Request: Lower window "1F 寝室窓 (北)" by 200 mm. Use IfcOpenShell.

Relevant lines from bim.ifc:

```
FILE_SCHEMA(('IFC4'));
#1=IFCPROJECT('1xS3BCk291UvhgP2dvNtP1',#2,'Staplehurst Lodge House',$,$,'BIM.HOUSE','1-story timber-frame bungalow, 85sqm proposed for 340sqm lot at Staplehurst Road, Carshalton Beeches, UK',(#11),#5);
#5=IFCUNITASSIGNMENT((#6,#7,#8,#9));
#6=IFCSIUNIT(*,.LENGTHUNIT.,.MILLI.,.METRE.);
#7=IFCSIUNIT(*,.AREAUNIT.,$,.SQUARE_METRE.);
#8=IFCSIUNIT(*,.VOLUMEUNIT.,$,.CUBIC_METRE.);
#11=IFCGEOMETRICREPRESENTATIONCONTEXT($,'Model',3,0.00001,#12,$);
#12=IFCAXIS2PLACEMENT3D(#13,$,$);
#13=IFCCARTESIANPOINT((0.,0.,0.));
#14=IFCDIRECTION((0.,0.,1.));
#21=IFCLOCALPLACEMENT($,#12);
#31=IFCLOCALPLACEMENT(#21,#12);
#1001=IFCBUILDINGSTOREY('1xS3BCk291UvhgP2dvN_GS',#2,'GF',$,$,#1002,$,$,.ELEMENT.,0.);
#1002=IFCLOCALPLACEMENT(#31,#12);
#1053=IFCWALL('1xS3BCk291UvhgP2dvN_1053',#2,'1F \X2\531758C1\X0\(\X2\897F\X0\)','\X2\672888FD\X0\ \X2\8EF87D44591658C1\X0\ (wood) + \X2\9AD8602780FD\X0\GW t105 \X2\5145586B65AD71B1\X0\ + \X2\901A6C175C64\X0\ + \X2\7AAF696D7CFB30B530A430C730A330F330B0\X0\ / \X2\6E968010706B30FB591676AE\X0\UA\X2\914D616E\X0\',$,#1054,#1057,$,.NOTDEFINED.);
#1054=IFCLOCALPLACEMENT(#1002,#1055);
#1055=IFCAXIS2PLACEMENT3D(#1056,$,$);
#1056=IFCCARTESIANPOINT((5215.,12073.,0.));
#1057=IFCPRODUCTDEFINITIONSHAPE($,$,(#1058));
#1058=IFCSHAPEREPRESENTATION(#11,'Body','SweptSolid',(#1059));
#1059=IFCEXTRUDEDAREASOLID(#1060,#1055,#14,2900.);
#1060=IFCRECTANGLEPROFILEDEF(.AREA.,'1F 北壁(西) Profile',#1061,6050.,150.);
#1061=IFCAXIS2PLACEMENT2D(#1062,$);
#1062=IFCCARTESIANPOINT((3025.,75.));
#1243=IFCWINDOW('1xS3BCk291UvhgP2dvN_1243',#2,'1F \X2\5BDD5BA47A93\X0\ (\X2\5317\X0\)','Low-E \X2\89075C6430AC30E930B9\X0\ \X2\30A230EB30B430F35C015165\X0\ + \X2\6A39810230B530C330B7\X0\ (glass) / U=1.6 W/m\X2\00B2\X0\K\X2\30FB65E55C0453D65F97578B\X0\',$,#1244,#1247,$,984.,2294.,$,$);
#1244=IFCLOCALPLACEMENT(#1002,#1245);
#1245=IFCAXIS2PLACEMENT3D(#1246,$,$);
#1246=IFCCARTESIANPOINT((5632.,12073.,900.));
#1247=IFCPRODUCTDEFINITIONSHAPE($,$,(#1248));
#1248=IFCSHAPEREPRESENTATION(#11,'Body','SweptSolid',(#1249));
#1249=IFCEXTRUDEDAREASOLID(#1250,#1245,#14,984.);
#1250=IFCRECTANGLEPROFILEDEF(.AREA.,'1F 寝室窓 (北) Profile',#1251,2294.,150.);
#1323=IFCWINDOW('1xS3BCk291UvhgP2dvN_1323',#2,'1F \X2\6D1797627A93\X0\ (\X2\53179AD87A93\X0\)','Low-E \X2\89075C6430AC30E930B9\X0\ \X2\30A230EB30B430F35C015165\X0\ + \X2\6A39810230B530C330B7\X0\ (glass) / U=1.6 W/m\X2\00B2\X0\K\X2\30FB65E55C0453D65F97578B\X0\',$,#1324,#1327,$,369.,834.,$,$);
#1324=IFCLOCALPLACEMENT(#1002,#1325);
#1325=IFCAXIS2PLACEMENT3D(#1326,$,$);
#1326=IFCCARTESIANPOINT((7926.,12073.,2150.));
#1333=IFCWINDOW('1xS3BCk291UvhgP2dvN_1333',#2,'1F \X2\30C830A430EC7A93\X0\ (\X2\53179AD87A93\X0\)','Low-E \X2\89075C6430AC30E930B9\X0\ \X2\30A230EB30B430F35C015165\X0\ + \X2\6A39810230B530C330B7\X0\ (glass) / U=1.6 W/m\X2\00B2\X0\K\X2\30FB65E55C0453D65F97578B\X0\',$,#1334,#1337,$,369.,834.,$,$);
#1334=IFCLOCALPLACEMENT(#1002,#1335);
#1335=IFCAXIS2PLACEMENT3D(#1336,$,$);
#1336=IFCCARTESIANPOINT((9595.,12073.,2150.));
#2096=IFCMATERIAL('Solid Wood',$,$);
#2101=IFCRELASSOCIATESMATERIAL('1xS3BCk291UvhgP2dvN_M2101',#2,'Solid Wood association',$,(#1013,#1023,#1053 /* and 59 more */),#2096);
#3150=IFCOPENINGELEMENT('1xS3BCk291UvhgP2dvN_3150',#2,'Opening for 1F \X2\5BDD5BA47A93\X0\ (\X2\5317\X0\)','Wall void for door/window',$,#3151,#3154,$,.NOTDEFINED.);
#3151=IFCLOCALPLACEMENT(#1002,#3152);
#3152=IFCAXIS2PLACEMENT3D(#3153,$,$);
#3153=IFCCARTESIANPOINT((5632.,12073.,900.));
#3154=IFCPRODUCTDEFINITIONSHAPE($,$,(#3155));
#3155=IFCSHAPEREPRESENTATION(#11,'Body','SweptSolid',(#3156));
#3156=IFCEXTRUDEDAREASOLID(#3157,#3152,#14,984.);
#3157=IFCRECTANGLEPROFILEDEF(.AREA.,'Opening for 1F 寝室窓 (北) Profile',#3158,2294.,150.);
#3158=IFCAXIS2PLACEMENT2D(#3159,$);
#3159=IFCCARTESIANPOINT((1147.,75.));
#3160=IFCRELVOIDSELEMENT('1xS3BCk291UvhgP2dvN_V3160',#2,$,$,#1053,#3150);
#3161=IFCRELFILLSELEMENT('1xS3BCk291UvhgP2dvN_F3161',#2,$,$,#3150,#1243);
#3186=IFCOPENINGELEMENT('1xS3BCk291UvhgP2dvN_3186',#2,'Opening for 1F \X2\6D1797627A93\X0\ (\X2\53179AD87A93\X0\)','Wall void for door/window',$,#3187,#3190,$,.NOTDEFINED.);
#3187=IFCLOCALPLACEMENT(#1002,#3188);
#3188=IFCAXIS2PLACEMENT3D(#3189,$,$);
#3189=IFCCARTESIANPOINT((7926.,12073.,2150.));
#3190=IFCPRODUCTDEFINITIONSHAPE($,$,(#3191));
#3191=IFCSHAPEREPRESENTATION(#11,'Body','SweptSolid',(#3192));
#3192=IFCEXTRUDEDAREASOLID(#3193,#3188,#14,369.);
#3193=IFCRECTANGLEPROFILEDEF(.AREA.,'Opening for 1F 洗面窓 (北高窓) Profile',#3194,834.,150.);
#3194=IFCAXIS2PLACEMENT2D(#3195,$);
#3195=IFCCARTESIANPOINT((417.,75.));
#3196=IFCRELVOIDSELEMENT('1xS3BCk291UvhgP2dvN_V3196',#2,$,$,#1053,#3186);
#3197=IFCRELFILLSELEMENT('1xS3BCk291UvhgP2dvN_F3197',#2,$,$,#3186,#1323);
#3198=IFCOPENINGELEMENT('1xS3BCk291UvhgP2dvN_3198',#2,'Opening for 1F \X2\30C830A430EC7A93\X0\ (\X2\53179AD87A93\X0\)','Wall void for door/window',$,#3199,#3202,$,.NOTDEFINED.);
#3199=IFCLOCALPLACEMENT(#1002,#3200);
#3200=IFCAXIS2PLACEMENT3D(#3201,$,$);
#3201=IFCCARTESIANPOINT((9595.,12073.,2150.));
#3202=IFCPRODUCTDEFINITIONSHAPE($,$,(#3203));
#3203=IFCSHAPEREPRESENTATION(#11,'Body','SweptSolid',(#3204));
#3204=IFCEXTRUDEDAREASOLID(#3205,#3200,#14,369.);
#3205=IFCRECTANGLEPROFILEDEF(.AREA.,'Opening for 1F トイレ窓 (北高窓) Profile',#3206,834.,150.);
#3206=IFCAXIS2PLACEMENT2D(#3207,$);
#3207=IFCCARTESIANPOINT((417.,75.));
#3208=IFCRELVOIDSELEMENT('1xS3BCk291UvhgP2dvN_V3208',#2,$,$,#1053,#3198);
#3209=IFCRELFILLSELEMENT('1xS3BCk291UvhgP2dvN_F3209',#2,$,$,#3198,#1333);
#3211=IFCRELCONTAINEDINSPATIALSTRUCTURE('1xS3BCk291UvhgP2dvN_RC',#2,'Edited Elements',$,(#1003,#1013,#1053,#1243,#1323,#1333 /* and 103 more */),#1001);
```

```python
import numpy as np
import ifcopenshell
import ifcopenshell.api.geometry
import ifcopenshell.util.placement
import ifcopenshell.util.unit

model = ifcopenshell.open("bim.ifc")
unit_scale = ifcopenshell.util.unit.calculate_unit_scale(model)

window = model.by_guid("1xS3BCk291UvhgP2dvN_1243")
opening = window.FillsVoids[0].RelatingOpeningElement
dz = -0.2 / unit_scale

shift = np.array([0.0, 0.0, dz])
# The window is not placed relative to its opening, so move both.
for product in (opening, window):
    matrix = ifcopenshell.util.placement.get_local_placement(product.ObjectPlacement)
    matrix[:3, 3] += shift
    ifcopenshell.api.geometry.edit_object_placement(model, product=product, matrix=matrix, is_si=False)

print(f"moved by {dz * unit_scale:+.3f} m")

model.write("bim-out.ifc")
```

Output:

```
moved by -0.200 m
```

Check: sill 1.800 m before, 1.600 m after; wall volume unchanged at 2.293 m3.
